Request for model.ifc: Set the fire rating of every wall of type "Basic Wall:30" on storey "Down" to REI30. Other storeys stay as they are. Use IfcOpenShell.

First a look at what the model holds.

```python
import ifcopenshell
import ifcopenshell.util.element

model = ifcopenshell.open("model.ifc")
print(model.schema)
storey = next(s for s in model.by_type("IfcBuildingStorey") if s.Name == "Down")
walls = [e for e in ifcopenshell.util.element.get_decomposition(storey) if e.is_a("IfcWall")]
seen = {}
for e in walls:
    element_type = ifcopenshell.util.element.get_type(e)
    key = (element_type.Name if element_type != e and element_type else None, ifcopenshell.util.element.get_pset(e, "Pset_WallCommon", "FireRating"))
    seen[key] = seen.get(key, 0) + 1
for (name, value), count in sorted(seen.items(), key=str):
    print(count, "x", name, "|", value)
```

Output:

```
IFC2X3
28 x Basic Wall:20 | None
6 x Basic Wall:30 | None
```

```python
import ifcopenshell
import ifcopenshell.api.pset
import ifcopenshell.util.element

model = ifcopenshell.open("model.ifc")

storey = next(s for s in model.by_type("IfcBuildingStorey") if s.Name == "Down")
walls = [e for e in ifcopenshell.util.element.get_decomposition(storey) if e.is_a("IfcWall")]

count = 0
for e in walls:
    element_type = ifcopenshell.util.element.get_type(e)
    if element_type in (None, e) or element_type.Name != "Basic Wall:30":
        continue
    # add_pset returns the element's existing set when there is one.
    pset = ifcopenshell.api.pset.add_pset(model, product=e, name="Pset_WallCommon")
    ifcopenshell.api.pset.edit_pset(model, pset=pset, properties={"FireRating": "REI30"})
    count += 1

print(count, "walls updated")

model.write("model_v2.ifc")
```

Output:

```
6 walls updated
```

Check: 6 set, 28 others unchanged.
